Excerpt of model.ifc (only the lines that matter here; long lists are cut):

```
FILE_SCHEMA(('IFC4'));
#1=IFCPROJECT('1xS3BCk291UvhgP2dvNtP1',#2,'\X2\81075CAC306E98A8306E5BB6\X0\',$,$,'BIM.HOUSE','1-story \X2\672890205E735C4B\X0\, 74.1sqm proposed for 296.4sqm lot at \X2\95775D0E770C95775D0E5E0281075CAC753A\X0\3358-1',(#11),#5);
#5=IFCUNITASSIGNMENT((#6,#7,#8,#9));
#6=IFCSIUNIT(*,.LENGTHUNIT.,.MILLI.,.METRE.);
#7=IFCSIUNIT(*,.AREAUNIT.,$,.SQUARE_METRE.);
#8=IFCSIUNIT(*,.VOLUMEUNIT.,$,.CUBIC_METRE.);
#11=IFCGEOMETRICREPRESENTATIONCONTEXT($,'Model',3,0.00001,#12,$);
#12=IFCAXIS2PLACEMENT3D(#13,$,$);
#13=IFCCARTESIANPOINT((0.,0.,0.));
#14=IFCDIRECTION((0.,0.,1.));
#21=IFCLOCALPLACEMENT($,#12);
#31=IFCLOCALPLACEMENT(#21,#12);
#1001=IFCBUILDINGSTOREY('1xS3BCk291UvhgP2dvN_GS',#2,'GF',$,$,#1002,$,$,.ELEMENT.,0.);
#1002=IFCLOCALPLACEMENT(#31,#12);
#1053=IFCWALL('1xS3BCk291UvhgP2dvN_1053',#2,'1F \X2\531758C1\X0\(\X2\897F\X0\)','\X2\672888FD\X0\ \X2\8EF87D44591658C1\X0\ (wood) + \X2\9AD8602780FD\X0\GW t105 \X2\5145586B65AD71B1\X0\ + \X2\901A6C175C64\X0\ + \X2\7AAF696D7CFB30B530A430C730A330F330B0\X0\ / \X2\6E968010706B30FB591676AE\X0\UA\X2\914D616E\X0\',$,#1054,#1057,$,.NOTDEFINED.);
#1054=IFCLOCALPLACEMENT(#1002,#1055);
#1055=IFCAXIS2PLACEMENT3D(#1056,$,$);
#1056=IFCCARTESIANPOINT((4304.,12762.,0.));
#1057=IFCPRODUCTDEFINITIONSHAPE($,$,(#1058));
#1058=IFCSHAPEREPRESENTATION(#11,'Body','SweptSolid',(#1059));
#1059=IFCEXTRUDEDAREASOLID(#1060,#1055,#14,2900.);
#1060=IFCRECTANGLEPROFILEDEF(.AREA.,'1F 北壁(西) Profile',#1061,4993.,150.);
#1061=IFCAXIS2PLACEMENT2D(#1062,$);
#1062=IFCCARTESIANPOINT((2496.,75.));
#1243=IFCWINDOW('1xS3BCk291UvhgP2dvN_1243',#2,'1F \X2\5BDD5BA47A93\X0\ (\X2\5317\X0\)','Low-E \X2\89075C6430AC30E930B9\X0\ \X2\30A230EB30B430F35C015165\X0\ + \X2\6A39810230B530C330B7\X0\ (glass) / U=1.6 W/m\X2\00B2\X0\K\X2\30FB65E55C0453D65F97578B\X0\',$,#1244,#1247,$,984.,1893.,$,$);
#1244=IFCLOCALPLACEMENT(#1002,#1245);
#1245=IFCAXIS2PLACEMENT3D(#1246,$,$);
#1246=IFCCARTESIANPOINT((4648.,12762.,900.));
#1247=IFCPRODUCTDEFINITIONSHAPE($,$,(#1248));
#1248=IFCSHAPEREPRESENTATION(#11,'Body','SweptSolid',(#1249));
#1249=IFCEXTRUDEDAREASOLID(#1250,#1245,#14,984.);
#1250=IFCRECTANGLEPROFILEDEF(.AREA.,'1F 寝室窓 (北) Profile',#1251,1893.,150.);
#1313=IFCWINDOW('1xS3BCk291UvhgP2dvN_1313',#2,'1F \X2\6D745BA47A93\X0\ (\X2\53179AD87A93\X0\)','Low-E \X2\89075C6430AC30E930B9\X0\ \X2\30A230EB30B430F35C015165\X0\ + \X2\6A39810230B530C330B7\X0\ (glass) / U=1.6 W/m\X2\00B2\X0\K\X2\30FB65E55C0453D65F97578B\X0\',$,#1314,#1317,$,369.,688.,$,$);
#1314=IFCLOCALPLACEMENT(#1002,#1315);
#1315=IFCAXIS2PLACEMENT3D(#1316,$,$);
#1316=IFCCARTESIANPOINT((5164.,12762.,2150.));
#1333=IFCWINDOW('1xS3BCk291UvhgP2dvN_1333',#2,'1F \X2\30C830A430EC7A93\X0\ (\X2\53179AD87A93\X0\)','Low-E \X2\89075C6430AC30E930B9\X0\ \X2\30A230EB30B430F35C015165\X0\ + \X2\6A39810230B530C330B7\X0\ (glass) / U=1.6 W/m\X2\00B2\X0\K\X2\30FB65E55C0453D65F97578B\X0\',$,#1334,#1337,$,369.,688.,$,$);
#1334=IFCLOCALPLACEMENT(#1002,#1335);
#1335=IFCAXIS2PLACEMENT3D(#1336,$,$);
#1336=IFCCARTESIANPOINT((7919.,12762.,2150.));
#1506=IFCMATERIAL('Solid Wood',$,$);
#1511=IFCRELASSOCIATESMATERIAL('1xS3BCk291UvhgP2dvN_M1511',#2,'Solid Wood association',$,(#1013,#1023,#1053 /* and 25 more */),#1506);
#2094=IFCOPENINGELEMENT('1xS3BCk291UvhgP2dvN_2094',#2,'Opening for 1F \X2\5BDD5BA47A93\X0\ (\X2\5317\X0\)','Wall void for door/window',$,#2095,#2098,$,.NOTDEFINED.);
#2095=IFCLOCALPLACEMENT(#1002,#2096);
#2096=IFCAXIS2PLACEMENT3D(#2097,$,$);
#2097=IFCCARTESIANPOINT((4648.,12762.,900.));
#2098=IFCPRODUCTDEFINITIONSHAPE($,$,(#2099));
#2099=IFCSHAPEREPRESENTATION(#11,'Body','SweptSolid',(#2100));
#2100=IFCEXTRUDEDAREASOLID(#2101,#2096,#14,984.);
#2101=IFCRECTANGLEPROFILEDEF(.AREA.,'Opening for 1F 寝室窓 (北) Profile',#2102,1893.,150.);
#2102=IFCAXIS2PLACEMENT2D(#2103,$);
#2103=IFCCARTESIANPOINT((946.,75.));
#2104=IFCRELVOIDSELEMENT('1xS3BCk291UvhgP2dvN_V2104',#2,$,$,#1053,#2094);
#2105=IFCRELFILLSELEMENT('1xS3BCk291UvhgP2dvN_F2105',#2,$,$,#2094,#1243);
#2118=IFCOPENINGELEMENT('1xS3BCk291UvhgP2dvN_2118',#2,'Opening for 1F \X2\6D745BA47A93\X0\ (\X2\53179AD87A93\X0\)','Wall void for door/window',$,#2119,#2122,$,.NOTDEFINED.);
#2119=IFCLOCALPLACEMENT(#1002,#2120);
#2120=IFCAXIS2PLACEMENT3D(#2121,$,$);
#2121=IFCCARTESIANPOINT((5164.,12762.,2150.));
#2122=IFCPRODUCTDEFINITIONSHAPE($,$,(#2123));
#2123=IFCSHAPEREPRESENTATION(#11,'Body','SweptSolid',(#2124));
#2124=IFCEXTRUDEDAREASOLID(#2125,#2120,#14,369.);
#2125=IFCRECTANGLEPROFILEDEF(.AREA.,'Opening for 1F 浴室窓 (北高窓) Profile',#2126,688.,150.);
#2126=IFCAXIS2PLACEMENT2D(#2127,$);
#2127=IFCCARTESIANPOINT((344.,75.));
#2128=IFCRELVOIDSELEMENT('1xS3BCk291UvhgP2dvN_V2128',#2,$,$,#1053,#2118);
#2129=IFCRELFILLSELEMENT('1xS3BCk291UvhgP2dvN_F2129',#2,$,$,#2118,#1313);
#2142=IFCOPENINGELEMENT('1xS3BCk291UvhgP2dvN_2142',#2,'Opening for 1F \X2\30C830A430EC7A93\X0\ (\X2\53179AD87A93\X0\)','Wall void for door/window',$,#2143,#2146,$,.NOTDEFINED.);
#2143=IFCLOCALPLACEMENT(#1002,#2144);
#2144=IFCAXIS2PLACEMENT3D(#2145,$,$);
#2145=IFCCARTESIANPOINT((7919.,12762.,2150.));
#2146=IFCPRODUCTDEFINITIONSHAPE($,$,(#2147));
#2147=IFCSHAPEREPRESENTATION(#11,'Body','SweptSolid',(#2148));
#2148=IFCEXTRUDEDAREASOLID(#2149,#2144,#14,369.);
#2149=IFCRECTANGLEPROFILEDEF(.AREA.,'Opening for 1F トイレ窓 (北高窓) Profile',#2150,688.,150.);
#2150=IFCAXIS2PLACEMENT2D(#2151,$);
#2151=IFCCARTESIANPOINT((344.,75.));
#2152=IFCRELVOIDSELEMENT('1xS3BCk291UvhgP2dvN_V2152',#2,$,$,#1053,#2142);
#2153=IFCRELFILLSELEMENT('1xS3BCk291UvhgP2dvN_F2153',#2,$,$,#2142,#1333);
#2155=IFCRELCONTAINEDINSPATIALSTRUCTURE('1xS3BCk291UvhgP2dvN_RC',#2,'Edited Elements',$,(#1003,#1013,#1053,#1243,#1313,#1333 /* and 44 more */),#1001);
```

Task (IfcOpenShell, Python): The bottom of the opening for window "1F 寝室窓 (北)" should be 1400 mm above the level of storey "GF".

```python
import numpy as np
import ifcopenshell
import ifcopenshell.api.geometry
import ifcopenshell.geom
import ifcopenshell.util.element
import ifcopenshell.util.placement
import ifcopenshell.util.shape
import ifcopenshell.util.unit

model = ifcopenshell.open("model.ifc")
unit_scale = ifcopenshell.util.unit.calculate_unit_scale(model)

window = model.by_guid("1xS3BCk291UvhgP2dvN_1243")
opening = window.FillsVoids[0].RelatingOpeningElement
storey = ifcopenshell.util.element.get_container(window, ifc_class="IfcBuildingStorey")
level = ifcopenshell.util.placement.get_local_placement(storey.ObjectPlacement)[2, 3]

# The opening's origin need not be at the sill, so measure its lowest point.
shape = ifcopenshell.geom.create_shape(ifcopenshell.geom.settings(), opening)
bottom = ifcopenshell.util.shape.get_shape_bottom_elevation(shape, shape.geometry) / unit_scale
dz = level + 1.4 / unit_scale - bottom

shift = np.array([0.0, 0.0, dz])
# The window is not placed relative to its opening, so move both.
for product in (opening, window):
    matrix = ifcopenshell.util.placement.get_local_placement(product.ObjectPlacement)
    matrix[:3, 3] += shift
    ifcopenshell.api.geometry.edit_object_placement(model, product=product, matrix=matrix, is_si=False)

print(f"moved by {dz * unit_scale:+.3f} m")

model.write("model-out.ifc")
```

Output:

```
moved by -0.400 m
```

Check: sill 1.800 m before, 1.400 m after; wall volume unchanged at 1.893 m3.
